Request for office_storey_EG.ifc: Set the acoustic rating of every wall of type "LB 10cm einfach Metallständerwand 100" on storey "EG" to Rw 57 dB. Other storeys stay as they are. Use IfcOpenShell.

First a look at what the model holds.

```python
import ifcopenshell
import ifcopenshell.util.element

model = ifcopenshell.open("office_storey_EG.ifc")
print(model.schema)
storey = next(s for s in model.by_type("IfcBuildingStorey") if s.Name == "EG")
walls = [e for e in ifcopenshell.util.element.get_decomposition(storey) if e.is_a("IfcWall")]
seen = {}
for e in walls:
    element_type = ifcopenshell.util.element.get_type(e)
    key = (element_type.Name if element_type != e and element_type else None, ifcopenshell.util.element.get_pset(e, "Pset_WallCommon", "AcousticRating"))
    seen[key] = seen.get(key, 0) + 1
for (name, value), count in sorted(seen.items(), key=str):
    print(count, "x", name, "|", value)
```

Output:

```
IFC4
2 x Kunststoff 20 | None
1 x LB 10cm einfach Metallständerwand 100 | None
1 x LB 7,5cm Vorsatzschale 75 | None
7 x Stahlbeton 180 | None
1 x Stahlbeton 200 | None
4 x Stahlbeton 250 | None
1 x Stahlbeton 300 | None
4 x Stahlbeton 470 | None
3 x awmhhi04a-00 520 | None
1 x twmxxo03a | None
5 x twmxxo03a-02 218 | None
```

```python
import ifcopenshell
import ifcopenshell.api.pset
import ifcopenshell.util.element

model = ifcopenshell.open("office_storey_EG.ifc")

storey = next(s for s in model.by_type("IfcBuildingStorey") if s.Name == "EG")
walls = [e for e in ifcopenshell.util.element.get_decomposition(storey) if e.is_a("IfcWall")]

count = 0
for e in walls:
    element_type = ifcopenshell.util.element.get_type(e)
    if element_type in (None, e) or element_type.Name != "LB 10cm einfach Metallständerwand 100":
        continue
    # add_pset returns the element's existing set when there is one.
    pset = ifcopenshell.api.pset.add_pset(model, product=e, name="Pset_WallCommon")
    ifcopenshell.api.pset.edit_pset(model, pset=pset, properties={"AcousticRating": "Rw 57 dB"})
    count += 1

print(count, "walls updated")

model.write("office_storey_EG_updated.ifc")
```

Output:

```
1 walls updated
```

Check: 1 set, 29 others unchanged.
